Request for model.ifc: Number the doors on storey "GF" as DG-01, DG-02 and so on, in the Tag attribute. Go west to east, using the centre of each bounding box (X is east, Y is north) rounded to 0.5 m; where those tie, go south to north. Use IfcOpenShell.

First a look at what the model holds.

```python
import ifcopenshell
import ifcopenshell.util.element
import ifcopenshell.util.placement

model = ifcopenshell.open("model.ifc")
print(model.schema)
storey = next(s for s in model.by_type("IfcBuildingStorey") if s.Name == "GF")
doors = [e for e in ifcopenshell.util.element.get_decomposition(storey) if e.is_a("IfcDoor")]
for e in sorted(doors, key=lambda e: e.id()):
    origin = ifcopenshell.util.placement.get_local_placement(e.ObjectPlacement)[:3, 3]
    print(e.id(), e.Tag, e.Name, origin.round(2) + 0.0, sep=" | ")
```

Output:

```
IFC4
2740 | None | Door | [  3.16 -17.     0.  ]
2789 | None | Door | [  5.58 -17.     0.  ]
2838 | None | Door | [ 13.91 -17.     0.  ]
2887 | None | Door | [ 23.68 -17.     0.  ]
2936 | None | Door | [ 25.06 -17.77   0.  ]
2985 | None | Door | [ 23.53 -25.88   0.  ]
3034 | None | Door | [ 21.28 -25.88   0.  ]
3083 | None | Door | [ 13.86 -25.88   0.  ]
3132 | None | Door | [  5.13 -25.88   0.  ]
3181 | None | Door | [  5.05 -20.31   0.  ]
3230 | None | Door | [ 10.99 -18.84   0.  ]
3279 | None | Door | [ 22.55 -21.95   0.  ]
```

```python
import ifcopenshell
import ifcopenshell.geom
import ifcopenshell.util.element
import ifcopenshell.util.shape

model = ifcopenshell.open("model.ifc")
settings = ifcopenshell.geom.settings()
settings.set("use-world-coords", True)


def centre(element):
    shape = ifcopenshell.geom.create_shape(settings, element)
    return ifcopenshell.util.shape.get_bbox_centroid(shape.geometry)


storey = next(s for s in model.by_type("IfcBuildingStorey") if s.Name == "GF")
doors = [e for e in ifcopenshell.util.element.get_decomposition(storey) if e.is_a("IfcDoor")]

# Insertion points can sit at a corner or the storey origin, so sort by the geometry (in metres).
centres = {e: centre(e) for e in doors}
doors.sort(key=lambda e: (round(centres[e][0] / 0.5), centres[e][1]))

for i, e in enumerate(doors, start=1):
    number = f"DG-{i:02d}"
    e.Tag = number
    print(e.id(), number)

model.write("model_v2.ifc")
```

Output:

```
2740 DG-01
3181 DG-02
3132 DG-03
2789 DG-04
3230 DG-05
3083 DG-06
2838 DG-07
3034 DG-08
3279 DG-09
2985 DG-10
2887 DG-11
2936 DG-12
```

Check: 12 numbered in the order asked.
